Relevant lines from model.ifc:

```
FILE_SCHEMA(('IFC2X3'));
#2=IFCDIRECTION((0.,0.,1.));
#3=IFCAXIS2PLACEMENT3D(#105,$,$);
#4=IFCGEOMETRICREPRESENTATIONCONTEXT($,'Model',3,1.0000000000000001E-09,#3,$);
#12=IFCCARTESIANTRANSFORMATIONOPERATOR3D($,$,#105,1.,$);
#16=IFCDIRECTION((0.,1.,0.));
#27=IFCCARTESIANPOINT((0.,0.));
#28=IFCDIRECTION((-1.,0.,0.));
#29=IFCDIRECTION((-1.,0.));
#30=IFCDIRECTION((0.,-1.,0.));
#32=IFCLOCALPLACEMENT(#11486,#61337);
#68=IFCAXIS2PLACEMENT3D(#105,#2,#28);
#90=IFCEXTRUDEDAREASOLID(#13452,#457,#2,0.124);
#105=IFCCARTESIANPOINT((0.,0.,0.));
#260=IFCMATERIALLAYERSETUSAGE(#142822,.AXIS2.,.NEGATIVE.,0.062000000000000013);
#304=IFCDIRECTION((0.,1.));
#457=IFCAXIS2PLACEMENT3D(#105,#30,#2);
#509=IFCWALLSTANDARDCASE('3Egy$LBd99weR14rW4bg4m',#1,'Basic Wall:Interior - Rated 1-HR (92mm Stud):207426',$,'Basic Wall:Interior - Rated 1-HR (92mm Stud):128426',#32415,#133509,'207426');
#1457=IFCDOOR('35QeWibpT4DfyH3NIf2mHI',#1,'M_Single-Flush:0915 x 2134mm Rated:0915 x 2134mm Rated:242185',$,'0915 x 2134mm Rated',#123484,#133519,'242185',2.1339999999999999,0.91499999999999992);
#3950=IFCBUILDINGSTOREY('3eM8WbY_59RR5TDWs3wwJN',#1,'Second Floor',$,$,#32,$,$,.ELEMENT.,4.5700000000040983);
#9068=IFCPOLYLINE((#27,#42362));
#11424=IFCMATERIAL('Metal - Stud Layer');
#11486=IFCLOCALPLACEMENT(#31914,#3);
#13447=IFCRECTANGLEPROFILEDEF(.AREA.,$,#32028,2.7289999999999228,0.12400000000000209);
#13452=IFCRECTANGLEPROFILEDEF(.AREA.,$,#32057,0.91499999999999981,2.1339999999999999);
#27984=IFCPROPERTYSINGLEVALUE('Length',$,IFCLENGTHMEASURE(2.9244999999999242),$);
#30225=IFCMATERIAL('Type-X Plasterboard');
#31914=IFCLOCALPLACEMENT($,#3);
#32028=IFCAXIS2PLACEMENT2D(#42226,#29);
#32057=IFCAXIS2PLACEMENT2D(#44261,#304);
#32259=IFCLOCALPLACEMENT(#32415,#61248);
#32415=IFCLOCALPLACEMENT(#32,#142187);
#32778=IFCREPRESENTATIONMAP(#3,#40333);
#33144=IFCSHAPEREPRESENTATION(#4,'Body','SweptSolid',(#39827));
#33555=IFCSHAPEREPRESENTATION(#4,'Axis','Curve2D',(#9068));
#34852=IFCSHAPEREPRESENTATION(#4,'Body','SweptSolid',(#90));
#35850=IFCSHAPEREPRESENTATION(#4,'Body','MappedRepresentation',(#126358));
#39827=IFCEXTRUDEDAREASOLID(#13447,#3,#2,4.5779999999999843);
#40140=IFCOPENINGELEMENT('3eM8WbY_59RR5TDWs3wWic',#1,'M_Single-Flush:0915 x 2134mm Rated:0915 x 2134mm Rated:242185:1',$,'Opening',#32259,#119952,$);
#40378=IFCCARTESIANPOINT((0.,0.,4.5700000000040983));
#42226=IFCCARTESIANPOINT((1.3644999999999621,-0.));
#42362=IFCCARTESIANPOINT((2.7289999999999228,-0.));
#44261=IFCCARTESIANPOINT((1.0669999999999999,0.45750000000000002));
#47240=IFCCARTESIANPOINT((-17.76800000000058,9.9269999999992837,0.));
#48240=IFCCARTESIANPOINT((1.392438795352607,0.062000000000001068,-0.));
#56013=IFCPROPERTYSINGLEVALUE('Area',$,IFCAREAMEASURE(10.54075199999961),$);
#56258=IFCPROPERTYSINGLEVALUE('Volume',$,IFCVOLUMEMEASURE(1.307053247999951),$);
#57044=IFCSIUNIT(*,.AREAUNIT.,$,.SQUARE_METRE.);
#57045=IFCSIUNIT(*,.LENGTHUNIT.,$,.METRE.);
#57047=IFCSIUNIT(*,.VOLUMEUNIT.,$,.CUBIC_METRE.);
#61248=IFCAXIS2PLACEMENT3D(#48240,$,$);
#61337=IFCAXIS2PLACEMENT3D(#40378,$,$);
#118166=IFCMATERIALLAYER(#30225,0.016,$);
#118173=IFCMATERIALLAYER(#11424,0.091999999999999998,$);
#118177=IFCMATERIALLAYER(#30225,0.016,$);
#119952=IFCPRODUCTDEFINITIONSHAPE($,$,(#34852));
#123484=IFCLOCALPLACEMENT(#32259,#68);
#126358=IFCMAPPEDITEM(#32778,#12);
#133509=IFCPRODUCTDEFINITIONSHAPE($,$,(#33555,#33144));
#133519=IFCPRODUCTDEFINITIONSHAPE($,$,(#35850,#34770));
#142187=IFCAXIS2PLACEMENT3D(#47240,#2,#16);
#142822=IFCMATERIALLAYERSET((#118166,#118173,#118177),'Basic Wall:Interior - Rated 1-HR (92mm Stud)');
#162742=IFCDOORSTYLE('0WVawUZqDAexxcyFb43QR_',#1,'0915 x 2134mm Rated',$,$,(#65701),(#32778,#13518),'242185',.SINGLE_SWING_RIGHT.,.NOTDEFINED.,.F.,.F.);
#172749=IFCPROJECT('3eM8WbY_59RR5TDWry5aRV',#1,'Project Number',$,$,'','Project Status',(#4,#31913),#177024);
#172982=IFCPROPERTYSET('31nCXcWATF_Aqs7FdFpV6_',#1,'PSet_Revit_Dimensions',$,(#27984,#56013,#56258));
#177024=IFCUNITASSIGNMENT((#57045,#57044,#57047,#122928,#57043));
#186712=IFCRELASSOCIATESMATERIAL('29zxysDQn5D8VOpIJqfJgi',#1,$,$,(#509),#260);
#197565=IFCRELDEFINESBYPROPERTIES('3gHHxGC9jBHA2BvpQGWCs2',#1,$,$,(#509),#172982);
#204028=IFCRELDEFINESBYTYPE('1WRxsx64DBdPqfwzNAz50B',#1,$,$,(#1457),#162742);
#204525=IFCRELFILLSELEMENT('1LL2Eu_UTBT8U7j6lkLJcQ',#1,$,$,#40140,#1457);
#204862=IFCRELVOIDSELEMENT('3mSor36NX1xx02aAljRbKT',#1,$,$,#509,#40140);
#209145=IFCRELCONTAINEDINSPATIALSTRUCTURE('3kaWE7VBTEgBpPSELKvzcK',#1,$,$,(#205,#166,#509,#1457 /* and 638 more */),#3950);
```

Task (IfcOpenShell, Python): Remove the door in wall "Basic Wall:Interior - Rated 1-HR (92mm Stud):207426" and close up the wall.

```python
import ifcopenshell
import ifcopenshell.api.feature
import ifcopenshell.api.pset
import ifcopenshell.api.root
import ifcopenshell.geom
import ifcopenshell.util.element
import ifcopenshell.util.shape
import ifcopenshell.util.unit

model = ifcopenshell.open("model.ifc")
area_scale = ifcopenshell.util.unit.calculate_unit_scale(model, "AREAUNIT")
volume_scale = ifcopenshell.util.unit.calculate_unit_scale(model, "VOLUMEUNIT")
settings = ifcopenshell.geom.settings()


def volume(element):
    """Net volume in cubic metres, openings subtracted."""
    shape = ifcopenshell.geom.create_shape(settings, element)
    return ifcopenshell.util.shape.get_volume(shape.geometry)


door = model.by_id(1457)
opening = door.FillsVoids[0].RelatingOpeningElement
wall = opening.VoidsElements[0].RelatingBuildingElement
before = volume(wall)

ifcopenshell.api.root.remove_product(model, product=door)
ifcopenshell.api.feature.remove_feature(model, feature=opening)

after = volume(wall)
thickness = 0.124  # wall thickness in metres

# Update the wall's stored quantities.
pset = model.by_id(ifcopenshell.util.element.get_pset(wall, "PSet_Revit_Dimensions", should_inherit=False)["id"])
ifcopenshell.api.pset.edit_pset(model, pset=pset, properties={
    "Area": model.create_entity("IfcAreaMeasure", after / thickness / area_scale),
    "Volume": model.create_entity("IfcVolumeMeasure", after / volume_scale),
})

print(f"wall volume {before:.3f} -> {after:.3f} m3")

model.write("model_v2.ifc")
```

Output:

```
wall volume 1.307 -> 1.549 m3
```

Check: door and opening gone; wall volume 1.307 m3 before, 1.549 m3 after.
